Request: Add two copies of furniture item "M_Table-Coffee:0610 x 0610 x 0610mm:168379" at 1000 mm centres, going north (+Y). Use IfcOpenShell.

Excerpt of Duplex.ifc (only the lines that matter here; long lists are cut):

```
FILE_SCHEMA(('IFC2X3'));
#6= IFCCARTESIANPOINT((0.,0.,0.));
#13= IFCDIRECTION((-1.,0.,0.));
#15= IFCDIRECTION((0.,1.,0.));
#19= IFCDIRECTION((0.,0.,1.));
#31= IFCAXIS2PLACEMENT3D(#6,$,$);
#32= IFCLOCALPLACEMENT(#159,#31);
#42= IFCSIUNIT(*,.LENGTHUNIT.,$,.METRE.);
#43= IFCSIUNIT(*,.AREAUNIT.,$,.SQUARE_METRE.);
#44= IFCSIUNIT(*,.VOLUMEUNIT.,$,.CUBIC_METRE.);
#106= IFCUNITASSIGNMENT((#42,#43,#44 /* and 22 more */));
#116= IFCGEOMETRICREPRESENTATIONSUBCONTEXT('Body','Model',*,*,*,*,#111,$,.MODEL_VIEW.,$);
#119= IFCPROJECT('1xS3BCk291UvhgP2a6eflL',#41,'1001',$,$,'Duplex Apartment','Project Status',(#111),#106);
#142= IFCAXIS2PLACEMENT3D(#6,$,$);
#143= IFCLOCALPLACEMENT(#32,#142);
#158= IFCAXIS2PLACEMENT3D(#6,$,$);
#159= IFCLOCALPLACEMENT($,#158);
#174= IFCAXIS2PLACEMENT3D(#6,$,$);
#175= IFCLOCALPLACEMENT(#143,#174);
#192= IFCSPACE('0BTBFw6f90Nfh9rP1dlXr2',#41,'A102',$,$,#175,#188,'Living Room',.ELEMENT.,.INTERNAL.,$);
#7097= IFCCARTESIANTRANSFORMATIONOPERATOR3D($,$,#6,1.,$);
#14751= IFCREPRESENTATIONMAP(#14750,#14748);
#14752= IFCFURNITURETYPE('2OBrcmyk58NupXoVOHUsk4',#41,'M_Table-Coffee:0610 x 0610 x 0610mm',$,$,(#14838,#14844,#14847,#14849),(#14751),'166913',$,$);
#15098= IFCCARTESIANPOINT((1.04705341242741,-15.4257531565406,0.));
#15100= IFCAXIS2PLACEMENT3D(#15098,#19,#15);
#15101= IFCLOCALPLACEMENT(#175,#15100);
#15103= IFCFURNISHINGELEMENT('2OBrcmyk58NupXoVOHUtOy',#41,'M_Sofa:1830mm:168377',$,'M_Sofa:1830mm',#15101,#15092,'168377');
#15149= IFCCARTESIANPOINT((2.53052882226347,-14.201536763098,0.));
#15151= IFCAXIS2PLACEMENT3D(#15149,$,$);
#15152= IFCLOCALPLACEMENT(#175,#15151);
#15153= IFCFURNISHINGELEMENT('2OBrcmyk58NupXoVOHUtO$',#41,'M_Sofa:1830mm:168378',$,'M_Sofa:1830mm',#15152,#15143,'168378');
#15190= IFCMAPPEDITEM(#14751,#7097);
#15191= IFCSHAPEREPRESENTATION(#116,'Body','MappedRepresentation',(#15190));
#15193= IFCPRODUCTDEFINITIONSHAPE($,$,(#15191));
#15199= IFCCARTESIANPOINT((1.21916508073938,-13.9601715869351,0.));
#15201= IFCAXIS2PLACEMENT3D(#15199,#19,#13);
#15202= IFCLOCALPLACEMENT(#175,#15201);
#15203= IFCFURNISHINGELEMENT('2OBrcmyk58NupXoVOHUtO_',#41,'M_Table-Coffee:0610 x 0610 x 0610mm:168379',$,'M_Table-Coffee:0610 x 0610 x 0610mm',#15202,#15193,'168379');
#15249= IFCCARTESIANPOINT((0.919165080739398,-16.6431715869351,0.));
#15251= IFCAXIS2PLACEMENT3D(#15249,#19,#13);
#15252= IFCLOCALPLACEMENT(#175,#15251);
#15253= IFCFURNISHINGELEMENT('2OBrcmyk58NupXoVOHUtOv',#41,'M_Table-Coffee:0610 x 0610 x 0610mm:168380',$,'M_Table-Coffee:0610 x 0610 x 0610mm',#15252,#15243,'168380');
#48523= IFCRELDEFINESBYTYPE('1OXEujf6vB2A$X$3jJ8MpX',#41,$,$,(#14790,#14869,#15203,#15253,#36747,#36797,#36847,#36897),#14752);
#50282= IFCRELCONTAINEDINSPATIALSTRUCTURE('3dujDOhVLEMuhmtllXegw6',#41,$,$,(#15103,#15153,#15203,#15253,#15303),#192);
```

```python
import numpy as np
import ifcopenshell
import ifcopenshell.api.geometry
import ifcopenshell.api.root
import ifcopenshell.util.element
import ifcopenshell.util.placement

model = ifcopenshell.open("Duplex.ifc")


def reuse_history(source, copy):
    """copy_class also copies each property set's owner history, people and application; keep the originals."""
    for rel in copy.IsDefinedBy:
        if rel.is_a("IfcRelDefinesByProperties") and (history := rel.RelatingPropertyDefinition.OwnerHistory):
            rel.RelatingPropertyDefinition.OwnerHistory = source.OwnerHistory
            ifcopenshell.util.element.remove_deep2(model, history)


source = model.by_guid("2OBrcmyk58NupXoVOHUtO_")
base = ifcopenshell.util.placement.get_local_placement(source.ObjectPlacement)
step = np.array([0.0, 1.0, 0.0]) * 1.0

for i in range(1, 3):
    copy = ifcopenshell.api.root.copy_class(model, product=source)
    copy.Representation = ifcopenshell.util.element.copy_deep(
        model, source.Representation, exclude=["IfcGeometricRepresentationContext", "IfcRepresentationMap"]
    )
    copy.Name = "M_Table-Coffee:0610 x 0610 x 0610mm"
    copy.Tag = None
    reuse_history(source, copy)
    matrix = base.copy()
    matrix[:3, 3] += i * step
    print("added at", matrix[:3, 3].round(3) + 0.0)
    ifcopenshell.api.geometry.edit_object_placement(model, product=copy, matrix=matrix, is_si=False)

model.write("Duplex-out.ifc")
```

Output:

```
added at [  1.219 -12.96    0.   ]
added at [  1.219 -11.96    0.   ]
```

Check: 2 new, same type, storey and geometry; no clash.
